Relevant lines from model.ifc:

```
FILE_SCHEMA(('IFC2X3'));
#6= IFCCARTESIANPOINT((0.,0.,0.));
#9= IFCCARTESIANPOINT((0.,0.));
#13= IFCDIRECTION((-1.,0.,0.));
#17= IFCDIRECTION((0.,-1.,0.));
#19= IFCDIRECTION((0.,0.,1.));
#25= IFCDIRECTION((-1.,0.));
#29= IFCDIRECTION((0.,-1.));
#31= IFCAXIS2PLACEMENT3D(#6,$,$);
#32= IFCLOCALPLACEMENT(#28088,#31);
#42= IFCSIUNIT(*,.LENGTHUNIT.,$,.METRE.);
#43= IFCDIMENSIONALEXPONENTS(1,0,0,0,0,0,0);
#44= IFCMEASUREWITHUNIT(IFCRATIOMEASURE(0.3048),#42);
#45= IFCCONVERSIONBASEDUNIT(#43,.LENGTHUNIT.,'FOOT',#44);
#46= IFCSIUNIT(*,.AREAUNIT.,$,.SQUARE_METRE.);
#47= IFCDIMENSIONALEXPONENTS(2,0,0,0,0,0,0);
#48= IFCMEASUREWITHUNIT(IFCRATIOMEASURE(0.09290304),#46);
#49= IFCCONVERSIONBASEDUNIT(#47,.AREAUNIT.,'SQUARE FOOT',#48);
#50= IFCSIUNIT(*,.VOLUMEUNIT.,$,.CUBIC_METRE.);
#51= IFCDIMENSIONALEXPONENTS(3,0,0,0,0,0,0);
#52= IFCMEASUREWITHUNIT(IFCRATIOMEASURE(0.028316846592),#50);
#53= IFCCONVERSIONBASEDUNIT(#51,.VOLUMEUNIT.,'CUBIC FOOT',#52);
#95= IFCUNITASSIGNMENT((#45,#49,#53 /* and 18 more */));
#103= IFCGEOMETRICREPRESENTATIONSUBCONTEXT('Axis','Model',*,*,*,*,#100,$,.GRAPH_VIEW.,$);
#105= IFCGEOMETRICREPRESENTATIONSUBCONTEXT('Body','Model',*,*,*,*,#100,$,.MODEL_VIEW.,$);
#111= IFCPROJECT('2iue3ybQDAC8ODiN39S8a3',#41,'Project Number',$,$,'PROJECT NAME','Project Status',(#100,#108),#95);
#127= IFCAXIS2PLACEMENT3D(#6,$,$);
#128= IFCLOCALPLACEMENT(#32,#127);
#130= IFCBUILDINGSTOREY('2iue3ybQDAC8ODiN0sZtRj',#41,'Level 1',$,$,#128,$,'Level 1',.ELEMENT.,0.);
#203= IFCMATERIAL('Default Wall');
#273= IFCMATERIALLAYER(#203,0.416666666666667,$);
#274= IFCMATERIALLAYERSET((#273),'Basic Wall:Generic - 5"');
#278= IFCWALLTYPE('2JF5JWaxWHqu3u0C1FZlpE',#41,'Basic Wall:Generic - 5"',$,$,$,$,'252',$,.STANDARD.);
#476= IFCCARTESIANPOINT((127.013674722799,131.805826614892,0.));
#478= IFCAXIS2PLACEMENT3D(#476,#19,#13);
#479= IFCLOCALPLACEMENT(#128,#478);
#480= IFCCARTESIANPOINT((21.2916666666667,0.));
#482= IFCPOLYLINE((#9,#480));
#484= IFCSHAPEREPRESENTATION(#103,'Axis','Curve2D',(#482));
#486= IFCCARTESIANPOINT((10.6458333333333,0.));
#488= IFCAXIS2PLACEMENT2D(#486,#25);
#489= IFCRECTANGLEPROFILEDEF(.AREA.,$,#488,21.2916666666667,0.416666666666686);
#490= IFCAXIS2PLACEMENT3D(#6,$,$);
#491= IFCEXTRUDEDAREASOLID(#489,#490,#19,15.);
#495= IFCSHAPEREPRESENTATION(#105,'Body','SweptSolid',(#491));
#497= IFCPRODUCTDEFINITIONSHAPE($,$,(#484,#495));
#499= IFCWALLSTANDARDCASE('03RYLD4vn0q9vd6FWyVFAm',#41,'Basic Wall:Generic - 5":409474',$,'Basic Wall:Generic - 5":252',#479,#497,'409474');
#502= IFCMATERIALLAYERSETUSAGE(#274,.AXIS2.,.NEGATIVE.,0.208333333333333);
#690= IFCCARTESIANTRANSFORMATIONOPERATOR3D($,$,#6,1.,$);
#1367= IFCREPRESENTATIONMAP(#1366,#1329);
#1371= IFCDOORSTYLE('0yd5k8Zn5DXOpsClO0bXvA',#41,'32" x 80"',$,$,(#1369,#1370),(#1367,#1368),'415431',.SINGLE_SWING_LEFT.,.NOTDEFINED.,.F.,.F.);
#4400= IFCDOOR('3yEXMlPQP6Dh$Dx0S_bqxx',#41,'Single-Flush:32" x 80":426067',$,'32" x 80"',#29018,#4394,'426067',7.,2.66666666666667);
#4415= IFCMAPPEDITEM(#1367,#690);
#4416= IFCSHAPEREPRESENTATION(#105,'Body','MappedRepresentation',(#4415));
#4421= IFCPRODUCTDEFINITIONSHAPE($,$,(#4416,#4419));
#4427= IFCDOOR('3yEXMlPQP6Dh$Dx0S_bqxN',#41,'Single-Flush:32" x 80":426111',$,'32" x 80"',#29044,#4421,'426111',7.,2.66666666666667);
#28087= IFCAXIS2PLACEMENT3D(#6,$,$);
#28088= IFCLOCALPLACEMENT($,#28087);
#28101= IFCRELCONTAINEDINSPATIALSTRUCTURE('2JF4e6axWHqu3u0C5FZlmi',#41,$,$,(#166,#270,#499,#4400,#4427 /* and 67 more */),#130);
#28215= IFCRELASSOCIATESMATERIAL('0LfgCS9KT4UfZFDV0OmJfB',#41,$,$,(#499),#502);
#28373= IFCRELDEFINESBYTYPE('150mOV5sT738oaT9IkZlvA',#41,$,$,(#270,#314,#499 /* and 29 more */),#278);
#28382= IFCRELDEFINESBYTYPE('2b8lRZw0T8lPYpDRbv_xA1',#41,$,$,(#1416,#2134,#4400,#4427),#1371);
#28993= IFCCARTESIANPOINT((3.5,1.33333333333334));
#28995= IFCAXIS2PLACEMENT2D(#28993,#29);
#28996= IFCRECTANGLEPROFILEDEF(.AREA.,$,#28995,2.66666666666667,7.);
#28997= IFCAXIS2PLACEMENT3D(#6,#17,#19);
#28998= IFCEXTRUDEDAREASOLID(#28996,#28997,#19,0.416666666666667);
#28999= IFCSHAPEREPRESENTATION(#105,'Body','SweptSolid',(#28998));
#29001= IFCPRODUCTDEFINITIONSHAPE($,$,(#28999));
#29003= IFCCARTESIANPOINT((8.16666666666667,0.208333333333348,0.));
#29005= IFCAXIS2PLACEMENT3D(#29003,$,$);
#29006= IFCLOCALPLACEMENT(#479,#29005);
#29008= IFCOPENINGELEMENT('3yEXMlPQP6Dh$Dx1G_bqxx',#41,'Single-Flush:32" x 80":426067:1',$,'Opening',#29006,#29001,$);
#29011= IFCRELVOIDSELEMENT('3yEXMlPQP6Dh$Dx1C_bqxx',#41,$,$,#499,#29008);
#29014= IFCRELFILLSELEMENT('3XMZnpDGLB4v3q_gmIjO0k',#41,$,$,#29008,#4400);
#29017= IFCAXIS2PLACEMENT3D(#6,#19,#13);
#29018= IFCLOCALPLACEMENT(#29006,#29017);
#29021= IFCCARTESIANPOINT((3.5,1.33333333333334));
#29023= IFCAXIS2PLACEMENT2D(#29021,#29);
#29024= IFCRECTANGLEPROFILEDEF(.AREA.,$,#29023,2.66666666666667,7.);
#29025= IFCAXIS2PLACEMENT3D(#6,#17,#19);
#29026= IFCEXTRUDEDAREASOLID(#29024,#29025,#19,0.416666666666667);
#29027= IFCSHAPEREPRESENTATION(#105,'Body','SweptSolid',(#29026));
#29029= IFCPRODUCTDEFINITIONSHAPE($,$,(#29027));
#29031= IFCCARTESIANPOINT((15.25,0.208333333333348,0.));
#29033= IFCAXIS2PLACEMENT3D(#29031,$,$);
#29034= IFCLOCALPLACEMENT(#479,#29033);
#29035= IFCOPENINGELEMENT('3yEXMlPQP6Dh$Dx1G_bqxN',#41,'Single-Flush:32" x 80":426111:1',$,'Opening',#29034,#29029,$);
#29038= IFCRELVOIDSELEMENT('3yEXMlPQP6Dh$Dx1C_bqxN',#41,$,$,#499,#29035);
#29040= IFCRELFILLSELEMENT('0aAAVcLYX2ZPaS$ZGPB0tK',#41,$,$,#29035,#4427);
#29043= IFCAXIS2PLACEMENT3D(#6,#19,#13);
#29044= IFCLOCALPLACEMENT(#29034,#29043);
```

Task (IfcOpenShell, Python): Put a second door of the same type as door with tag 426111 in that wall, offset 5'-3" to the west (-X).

```python
import ifcopenshell
import ifcopenshell.api.feature
import ifcopenshell.api.geometry
import ifcopenshell.api.root
import ifcopenshell.geom
import ifcopenshell.util.element
import ifcopenshell.util.placement
import ifcopenshell.util.shape
import ifcopenshell.util.unit

model = ifcopenshell.open("model.ifc")
unit_scale = ifcopenshell.util.unit.calculate_unit_scale(model)
settings = ifcopenshell.geom.settings()


def volume(element):
    """Net volume in cubic metres, openings subtracted."""
    shape = ifcopenshell.geom.create_shape(settings, element)
    return ifcopenshell.util.shape.get_volume(shape.geometry)


def reuse_history(source, copy):
    """copy_class also copies each property set's owner history, people and application; keep the originals."""
    for rel in copy.IsDefinedBy:
        if rel.is_a("IfcRelDefinesByProperties") and (history := rel.RelatingPropertyDefinition.OwnerHistory):
            rel.RelatingPropertyDefinition.OwnerHistory = source.OwnerHistory
            ifcopenshell.util.element.remove_deep2(model, history)


door = model.by_guid("3yEXMlPQP6Dh$Dx0S_bqxN")
opening = door.FillsVoids[0].RelatingOpeningElement
wall = opening.VoidsElements[0].RelatingBuildingElement
before = volume(wall)
shift = ifcopenshell.util.placement.get_local_placement(wall.ObjectPlacement)[:3, 0] * 63 * 0.0254 / unit_scale

# copy_class copies the void relationship, type, container and properties, but no geometry.
new_opening = ifcopenshell.api.root.copy_class(model, product=opening)
new_opening.Representation = ifcopenshell.util.element.copy_deep(
    model, opening.Representation, exclude=["IfcGeometricRepresentationContext", "IfcRepresentationMap"]
)
new_opening.Name = 'Single-Flush:32" x 80"'
new_door = ifcopenshell.api.root.copy_class(model, product=door)
new_door.Representation = ifcopenshell.util.element.copy_deep(
    model, door.Representation, exclude=["IfcGeometricRepresentationContext", "IfcRepresentationMap"]
)
new_door.Name = 'Single-Flush:32" x 80"'
new_door.Tag = None
reuse_history(door, new_door)
fills = ifcopenshell.api.feature.add_filling(model, opening=new_opening, element=new_door)
fills.OwnerHistory = new_door.OwnerHistory  # required in IFC2X3

for old, new in ((opening, new_opening), (door, new_door)):
    matrix = ifcopenshell.util.placement.get_local_placement(old.ObjectPlacement)
    matrix[:3, 3] += shift
    ifcopenshell.api.geometry.edit_object_placement(model, product=new, matrix=matrix, is_si=False)

after = volume(wall)

print(f"wall volume {before:.3f} -> {after:.3f} m3")

model.write("model-out.ifc")
```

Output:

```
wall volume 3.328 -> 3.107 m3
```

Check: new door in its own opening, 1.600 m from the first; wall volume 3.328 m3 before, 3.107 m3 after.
